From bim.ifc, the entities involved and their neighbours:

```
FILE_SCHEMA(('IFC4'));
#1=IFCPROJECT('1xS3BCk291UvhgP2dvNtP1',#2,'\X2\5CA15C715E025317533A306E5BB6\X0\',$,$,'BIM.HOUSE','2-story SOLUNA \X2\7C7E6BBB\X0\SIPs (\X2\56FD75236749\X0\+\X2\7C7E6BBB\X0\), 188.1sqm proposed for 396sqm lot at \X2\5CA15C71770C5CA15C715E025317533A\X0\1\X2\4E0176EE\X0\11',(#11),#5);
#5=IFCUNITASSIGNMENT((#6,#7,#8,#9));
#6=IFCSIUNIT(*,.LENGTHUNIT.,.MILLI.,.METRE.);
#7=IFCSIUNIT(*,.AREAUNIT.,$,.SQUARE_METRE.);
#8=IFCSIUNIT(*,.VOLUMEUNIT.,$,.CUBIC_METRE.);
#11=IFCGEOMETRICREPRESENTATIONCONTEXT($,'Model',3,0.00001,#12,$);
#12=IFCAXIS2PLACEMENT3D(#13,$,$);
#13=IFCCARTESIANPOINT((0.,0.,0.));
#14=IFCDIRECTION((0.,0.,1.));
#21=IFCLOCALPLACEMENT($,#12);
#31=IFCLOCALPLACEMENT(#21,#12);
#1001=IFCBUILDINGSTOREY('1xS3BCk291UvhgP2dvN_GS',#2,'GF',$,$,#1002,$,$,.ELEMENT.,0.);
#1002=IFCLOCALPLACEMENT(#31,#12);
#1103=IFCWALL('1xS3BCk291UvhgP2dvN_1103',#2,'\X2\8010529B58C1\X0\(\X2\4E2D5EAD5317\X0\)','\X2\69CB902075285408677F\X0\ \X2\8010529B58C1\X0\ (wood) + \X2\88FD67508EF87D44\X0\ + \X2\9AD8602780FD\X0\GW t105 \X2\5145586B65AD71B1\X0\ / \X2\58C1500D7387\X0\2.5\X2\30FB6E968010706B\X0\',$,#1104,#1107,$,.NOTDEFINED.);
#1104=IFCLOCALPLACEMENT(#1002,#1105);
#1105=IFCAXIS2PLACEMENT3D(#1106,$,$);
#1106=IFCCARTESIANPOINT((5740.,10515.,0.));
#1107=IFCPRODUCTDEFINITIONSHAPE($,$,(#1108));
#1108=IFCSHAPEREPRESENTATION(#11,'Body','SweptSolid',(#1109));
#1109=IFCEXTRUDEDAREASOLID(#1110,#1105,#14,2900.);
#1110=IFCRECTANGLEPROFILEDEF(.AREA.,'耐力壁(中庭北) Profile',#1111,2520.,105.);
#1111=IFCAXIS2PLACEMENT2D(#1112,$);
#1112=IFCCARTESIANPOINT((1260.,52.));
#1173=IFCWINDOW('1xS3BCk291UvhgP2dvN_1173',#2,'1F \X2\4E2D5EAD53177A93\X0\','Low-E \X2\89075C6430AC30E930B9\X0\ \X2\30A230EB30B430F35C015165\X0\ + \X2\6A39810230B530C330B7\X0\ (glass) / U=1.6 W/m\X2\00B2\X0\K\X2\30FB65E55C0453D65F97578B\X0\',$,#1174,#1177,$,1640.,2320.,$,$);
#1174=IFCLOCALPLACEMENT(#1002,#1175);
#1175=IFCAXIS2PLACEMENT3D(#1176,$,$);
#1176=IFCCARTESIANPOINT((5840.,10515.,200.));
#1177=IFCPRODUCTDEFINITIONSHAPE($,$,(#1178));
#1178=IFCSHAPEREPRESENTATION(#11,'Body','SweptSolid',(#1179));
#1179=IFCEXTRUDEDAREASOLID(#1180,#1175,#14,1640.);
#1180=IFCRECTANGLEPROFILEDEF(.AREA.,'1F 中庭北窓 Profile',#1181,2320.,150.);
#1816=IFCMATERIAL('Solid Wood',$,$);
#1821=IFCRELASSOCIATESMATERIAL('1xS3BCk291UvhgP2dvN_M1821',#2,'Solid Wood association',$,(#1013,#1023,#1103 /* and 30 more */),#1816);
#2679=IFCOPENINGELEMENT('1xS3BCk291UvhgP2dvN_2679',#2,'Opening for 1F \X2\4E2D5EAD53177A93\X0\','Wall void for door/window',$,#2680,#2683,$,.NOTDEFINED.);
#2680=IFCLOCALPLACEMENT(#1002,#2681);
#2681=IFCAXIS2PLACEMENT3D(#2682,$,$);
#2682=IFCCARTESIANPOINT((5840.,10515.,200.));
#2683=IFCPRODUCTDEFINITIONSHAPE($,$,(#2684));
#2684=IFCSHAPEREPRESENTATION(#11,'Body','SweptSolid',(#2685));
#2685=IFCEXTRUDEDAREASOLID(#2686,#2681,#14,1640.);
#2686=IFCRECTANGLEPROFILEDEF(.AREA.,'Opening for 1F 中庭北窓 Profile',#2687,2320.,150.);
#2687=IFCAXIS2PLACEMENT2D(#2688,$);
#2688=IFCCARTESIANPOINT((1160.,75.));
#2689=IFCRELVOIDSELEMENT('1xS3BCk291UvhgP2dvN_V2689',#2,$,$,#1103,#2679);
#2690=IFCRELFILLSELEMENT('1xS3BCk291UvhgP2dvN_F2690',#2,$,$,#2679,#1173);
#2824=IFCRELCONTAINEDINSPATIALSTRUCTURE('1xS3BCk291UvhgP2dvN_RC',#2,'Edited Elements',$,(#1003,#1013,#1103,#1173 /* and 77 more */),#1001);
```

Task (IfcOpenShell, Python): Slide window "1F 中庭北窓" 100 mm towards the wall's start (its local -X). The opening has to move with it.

```python
import ifcopenshell
import ifcopenshell.api.geometry
import ifcopenshell.util.placement
import ifcopenshell.util.unit

model = ifcopenshell.open("bim.ifc")
unit_scale = ifcopenshell.util.unit.calculate_unit_scale(model)

window = model.by_guid("1xS3BCk291UvhgP2dvN_1173")
opening = window.FillsVoids[0].RelatingOpeningElement
wall = opening.VoidsElements[0].RelatingBuildingElement

wall_matrix = ifcopenshell.util.placement.get_local_placement(wall.ObjectPlacement)
shift = wall_matrix[:3, 0] * -0.1 / unit_scale
before = ifcopenshell.util.placement.get_local_placement(window.ObjectPlacement)[:3, 3].copy()

# The window is not placed relative to its opening, so move both.
for product in (opening, window):
    matrix = ifcopenshell.util.placement.get_local_placement(product.ObjectPlacement)
    matrix[:3, 3] += shift
    ifcopenshell.api.geometry.edit_object_placement(model, product=product, matrix=matrix, is_si=False)

after = ifcopenshell.util.placement.get_local_placement(window.ObjectPlacement)[:3, 3]
print("window moved by", (after - before).round(3) + 0.0)

model.write("bim_rev.ifc")
```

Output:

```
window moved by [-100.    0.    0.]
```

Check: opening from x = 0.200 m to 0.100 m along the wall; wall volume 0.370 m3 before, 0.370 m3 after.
